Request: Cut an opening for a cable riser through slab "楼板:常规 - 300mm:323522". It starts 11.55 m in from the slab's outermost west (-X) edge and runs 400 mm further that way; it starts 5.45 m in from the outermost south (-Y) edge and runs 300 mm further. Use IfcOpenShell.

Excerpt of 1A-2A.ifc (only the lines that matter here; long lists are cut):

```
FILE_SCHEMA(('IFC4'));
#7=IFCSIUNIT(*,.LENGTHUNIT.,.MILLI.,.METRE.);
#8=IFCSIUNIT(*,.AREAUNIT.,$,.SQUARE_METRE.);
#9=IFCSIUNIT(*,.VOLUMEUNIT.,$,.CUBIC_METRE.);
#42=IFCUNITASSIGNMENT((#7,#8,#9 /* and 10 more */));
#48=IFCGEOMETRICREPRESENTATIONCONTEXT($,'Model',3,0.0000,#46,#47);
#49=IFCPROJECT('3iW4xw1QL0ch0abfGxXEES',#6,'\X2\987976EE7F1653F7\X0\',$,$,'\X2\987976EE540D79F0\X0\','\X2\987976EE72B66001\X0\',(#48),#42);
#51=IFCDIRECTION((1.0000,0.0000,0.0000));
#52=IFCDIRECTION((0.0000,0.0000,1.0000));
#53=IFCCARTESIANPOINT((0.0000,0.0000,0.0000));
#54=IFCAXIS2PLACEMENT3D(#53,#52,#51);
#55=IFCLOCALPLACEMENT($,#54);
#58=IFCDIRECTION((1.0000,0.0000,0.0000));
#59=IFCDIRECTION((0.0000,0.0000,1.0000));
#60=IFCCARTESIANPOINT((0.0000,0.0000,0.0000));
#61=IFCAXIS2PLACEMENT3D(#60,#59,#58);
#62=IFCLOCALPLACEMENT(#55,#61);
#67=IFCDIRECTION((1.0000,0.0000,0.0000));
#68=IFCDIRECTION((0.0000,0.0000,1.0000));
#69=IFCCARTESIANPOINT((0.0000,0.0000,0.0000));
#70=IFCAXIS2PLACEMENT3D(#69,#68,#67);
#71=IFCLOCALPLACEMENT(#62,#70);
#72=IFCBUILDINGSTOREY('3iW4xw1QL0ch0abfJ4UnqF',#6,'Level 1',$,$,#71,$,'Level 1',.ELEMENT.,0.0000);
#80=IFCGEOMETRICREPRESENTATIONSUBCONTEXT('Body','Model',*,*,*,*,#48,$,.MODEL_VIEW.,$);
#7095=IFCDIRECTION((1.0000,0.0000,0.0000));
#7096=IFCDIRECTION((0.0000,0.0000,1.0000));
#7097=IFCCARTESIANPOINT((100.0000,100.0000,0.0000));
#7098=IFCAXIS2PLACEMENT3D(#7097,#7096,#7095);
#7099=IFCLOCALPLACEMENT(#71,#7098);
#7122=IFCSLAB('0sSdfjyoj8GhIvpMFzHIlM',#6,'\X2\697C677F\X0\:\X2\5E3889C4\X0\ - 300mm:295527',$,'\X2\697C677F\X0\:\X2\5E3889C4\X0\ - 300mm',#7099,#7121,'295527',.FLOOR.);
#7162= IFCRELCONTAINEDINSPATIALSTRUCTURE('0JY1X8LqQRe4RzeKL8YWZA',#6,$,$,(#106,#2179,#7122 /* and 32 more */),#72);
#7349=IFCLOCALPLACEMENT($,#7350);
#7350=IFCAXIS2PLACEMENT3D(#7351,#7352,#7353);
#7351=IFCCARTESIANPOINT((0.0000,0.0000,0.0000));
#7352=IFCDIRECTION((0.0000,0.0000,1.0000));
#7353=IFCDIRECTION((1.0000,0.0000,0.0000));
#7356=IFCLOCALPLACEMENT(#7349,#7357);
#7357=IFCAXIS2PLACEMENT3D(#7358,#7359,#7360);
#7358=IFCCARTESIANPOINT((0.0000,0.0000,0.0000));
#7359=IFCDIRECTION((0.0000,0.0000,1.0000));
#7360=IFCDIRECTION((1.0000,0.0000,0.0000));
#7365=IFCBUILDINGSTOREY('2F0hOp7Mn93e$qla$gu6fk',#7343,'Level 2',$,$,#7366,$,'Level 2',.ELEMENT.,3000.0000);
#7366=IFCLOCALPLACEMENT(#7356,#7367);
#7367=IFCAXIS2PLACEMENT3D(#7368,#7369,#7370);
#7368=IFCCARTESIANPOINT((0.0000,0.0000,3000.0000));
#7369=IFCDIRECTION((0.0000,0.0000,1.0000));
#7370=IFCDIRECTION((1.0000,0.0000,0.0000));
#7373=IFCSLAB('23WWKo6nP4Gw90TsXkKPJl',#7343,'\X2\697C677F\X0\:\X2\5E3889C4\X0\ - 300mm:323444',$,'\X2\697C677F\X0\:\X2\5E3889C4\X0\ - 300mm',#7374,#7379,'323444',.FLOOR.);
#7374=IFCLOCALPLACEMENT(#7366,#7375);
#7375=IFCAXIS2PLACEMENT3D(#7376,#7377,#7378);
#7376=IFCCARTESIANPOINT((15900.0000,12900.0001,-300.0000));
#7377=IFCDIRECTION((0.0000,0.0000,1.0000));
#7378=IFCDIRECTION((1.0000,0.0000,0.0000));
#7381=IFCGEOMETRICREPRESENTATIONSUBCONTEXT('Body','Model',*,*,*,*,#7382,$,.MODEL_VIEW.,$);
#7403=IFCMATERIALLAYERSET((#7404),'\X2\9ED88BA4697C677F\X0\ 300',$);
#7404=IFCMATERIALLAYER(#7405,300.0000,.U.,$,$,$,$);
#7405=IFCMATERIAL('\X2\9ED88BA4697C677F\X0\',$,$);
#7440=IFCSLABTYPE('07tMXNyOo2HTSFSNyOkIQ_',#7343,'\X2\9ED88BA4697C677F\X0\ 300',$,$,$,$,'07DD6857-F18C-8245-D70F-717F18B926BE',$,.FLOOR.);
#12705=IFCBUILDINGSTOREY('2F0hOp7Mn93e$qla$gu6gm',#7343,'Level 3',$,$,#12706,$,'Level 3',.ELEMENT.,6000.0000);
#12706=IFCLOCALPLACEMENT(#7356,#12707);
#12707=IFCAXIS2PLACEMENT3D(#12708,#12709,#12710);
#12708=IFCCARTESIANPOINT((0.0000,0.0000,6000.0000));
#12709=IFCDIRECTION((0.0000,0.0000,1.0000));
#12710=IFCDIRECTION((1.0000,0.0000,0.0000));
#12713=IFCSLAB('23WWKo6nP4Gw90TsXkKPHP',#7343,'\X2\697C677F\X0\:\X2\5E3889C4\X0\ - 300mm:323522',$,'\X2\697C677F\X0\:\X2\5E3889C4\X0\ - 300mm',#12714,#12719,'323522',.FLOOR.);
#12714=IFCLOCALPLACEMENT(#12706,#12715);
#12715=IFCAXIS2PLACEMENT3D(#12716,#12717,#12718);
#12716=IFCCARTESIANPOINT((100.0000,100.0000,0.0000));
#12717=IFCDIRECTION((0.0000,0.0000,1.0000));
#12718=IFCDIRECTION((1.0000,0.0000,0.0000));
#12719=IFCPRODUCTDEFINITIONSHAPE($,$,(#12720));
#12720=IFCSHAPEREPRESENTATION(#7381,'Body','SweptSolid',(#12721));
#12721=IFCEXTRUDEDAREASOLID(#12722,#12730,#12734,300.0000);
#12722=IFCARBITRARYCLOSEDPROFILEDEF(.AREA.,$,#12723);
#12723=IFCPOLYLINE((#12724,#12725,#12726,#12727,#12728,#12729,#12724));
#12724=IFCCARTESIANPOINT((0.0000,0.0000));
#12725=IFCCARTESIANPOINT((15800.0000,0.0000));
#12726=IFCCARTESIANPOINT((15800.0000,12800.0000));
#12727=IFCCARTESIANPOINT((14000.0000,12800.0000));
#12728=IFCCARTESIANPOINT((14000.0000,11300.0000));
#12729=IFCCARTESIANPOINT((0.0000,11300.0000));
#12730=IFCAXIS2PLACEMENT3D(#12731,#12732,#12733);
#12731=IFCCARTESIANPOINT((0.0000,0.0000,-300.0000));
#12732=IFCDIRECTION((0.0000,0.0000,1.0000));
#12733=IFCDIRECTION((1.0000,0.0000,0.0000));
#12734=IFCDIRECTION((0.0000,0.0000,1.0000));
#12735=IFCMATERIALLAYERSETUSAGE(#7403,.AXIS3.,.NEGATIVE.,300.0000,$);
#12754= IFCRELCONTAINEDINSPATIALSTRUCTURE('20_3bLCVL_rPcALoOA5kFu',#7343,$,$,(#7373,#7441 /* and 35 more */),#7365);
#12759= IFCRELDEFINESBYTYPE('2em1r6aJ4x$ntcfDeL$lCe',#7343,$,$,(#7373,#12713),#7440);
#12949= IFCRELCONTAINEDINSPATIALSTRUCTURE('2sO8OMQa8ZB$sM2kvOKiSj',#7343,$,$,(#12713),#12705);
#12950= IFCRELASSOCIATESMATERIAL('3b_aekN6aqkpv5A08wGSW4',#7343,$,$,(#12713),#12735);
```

```python
import numpy as np
import ifcopenshell
import ifcopenshell.api.feature
import ifcopenshell.api.geometry
import ifcopenshell.api.root
import ifcopenshell.geom
import ifcopenshell.util.placement
import ifcopenshell.util.representation
import ifcopenshell.util.shape
import ifcopenshell.util.unit

model = ifcopenshell.open("1A-2A.ifc")
unit_scale = ifcopenshell.util.unit.calculate_unit_scale(model)
settings = ifcopenshell.geom.settings()


def volume(element):
    """Net volume in cubic metres, openings subtracted."""
    shape = ifcopenshell.geom.create_shape(settings, element)
    return ifcopenshell.util.shape.get_volume(shape.geometry)


slab = model.by_id(12713)
before = volume(slab)

# Extent in the slab's own axes, in metres. The edges named are its -X and -Y sides.
slab_shape = ifcopenshell.geom.create_shape(settings, slab)
vertices = ifcopenshell.util.shape.get_vertices(slab_shape.geometry)
x_min, y_min, bottom = vertices.min(axis=0)
top = vertices[:, 2].max()

opening = ifcopenshell.api.root.create_entity(model, ifc_class="IfcOpeningElement", name="Cable riser opening", predefined_type="OPENING")
context = ifcopenshell.util.representation.get_context(model, "Model", "Body", "MODEL_VIEW")
width, depth = 0.4, 0.3
outline = [(0.0, 0.0), (width, 0.0), (width, depth), (0.0, depth), (0.0, 0.0)]
# Overshoot both faces by 50 mm so the cut is clean.
shape = ifcopenshell.api.geometry.add_slab_representation(
    model, context=context, depth=top - bottom + 0.1, polyline=outline
)
ifcopenshell.api.geometry.assign_representation(model, product=opening, representation=shape)

matrix = ifcopenshell.util.placement.get_local_placement(slab.ObjectPlacement)
matrix[:, 3] = matrix @ np.append(np.array([x_min + 11.55, y_min + 5.45, bottom - 0.05]) / unit_scale, 1.0)
ifcopenshell.api.geometry.edit_object_placement(model, product=opening, matrix=matrix, is_si=False)
ifcopenshell.api.feature.add_feature(model, feature=opening, element=slab)

after = volume(slab)

print(f"slab volume {before:.3f} -> {after:.3f} m3")

model.write("1A-2A_rev.ifc")
```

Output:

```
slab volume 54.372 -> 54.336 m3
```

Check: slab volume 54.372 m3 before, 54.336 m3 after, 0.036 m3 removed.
